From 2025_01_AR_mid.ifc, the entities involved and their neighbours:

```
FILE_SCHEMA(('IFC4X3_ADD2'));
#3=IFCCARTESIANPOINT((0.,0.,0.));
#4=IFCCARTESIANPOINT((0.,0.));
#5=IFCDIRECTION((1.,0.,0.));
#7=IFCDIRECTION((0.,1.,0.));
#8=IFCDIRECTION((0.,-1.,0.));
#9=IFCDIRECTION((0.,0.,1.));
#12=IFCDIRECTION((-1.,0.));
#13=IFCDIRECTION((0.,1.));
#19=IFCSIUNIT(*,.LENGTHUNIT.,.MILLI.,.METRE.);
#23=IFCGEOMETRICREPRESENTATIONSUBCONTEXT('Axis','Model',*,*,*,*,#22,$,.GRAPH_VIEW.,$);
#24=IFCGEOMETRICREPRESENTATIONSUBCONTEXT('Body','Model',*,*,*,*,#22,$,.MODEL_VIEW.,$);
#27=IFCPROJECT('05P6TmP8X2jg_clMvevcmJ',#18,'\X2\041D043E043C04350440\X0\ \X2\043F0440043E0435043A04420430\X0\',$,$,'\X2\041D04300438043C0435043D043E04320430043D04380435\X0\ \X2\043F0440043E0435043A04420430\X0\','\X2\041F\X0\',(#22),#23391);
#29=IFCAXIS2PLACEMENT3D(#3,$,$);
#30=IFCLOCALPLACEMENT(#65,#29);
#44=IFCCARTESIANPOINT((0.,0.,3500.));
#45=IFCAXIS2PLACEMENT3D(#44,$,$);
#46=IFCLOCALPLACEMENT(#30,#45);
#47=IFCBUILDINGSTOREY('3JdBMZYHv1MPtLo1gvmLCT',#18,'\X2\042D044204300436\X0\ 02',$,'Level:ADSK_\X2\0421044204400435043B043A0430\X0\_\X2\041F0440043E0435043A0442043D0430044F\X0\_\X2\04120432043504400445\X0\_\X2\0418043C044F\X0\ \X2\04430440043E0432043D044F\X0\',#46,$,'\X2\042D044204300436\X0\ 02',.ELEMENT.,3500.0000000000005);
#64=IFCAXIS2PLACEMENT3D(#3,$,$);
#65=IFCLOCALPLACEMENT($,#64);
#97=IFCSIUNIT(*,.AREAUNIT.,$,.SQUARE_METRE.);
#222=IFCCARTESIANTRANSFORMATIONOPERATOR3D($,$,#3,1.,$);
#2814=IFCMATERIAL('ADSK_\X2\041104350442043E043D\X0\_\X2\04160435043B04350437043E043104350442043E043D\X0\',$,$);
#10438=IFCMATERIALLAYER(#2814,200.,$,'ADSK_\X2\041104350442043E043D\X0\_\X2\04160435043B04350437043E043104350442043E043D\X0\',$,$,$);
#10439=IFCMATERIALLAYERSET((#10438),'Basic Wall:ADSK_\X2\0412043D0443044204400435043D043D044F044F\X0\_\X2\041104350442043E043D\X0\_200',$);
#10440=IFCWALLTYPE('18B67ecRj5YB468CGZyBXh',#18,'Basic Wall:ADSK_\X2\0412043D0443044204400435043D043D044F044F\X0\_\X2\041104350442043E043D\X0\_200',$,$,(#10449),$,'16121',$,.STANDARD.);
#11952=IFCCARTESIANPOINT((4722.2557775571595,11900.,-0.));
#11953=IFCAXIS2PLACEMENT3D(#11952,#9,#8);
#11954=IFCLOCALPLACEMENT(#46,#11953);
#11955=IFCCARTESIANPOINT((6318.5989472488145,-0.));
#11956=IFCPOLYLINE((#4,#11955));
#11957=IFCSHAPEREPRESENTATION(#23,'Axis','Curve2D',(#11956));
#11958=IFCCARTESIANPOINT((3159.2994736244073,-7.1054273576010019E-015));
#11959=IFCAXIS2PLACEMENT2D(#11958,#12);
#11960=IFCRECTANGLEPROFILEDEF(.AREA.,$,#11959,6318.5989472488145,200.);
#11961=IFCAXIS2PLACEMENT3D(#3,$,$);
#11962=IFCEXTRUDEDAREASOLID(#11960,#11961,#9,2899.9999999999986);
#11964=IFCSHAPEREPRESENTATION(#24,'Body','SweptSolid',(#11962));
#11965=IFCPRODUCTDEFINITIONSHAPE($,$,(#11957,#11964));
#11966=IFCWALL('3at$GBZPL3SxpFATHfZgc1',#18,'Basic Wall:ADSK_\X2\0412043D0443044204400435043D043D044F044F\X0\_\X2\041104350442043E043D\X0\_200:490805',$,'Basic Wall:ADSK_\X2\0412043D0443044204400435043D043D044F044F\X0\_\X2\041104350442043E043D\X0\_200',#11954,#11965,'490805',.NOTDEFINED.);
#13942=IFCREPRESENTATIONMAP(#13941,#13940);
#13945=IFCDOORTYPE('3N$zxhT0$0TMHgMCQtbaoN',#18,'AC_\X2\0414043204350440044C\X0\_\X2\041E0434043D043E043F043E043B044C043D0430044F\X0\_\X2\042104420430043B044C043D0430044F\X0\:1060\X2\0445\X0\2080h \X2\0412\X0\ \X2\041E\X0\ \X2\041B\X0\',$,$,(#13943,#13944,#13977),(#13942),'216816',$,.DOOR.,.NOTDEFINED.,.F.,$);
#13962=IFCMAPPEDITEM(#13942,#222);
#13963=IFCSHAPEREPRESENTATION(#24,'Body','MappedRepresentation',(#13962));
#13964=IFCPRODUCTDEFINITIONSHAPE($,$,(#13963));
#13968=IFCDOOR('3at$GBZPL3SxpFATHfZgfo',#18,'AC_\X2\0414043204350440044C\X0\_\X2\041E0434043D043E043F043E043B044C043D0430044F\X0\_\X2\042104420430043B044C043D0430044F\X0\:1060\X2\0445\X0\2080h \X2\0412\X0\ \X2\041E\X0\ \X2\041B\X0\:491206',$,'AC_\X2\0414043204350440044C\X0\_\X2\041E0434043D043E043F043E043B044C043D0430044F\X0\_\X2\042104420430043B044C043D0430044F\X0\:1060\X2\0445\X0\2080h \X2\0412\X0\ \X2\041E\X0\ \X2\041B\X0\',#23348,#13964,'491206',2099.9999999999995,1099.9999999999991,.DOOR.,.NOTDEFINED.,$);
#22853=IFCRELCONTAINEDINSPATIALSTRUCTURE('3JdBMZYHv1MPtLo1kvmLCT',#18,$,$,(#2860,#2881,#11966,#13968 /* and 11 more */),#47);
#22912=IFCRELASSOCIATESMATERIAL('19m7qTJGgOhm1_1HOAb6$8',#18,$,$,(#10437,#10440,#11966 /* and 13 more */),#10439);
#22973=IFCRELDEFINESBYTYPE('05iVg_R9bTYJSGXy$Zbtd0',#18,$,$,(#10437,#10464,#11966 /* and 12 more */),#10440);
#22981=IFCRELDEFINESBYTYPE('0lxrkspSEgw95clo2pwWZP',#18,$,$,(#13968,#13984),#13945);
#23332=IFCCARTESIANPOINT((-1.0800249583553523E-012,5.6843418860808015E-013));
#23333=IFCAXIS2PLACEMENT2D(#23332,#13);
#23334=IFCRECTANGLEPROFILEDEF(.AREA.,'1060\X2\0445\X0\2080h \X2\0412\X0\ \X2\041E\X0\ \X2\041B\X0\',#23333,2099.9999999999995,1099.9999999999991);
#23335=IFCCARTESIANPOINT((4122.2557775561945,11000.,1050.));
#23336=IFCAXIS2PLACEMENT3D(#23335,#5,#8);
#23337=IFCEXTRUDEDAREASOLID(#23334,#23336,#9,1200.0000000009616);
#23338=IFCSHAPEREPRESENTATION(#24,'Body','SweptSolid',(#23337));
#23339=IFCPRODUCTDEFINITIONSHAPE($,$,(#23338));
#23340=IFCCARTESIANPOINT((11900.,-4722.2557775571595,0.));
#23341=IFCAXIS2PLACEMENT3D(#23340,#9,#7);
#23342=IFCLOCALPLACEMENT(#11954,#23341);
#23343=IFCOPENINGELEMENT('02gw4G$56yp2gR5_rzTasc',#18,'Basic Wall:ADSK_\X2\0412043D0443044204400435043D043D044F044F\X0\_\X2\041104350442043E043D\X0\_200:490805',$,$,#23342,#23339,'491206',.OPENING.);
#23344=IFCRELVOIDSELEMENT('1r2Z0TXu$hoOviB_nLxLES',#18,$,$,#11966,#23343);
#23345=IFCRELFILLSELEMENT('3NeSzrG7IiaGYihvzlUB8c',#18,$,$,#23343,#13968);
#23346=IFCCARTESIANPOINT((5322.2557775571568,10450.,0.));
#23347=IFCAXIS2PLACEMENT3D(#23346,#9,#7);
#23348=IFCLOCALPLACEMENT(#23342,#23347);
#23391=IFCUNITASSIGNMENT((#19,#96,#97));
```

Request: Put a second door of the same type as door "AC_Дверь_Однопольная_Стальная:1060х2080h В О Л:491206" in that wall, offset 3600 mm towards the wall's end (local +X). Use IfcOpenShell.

```python
import ifcopenshell
import ifcopenshell.api.feature
import ifcopenshell.api.geometry
import ifcopenshell.api.root
import ifcopenshell.geom
import ifcopenshell.util.element
import ifcopenshell.util.placement
import ifcopenshell.util.shape
import ifcopenshell.util.unit

model = ifcopenshell.open("2025_01_AR_mid.ifc")
unit_scale = ifcopenshell.util.unit.calculate_unit_scale(model)
settings = ifcopenshell.geom.settings()


def volume(element):
    """Net volume in cubic metres, openings subtracted."""
    shape = ifcopenshell.geom.create_shape(settings, element)
    return ifcopenshell.util.shape.get_volume(shape.geometry)


def reuse_history(source, copy):
    """copy_class also copies each property set's owner history, people and application; keep the originals."""
    for rel in copy.IsDefinedBy:
        if rel.is_a("IfcRelDefinesByProperties") and (history := rel.RelatingPropertyDefinition.OwnerHistory):
            rel.RelatingPropertyDefinition.OwnerHistory = source.OwnerHistory
            ifcopenshell.util.element.remove_deep2(model, history)


door = model.by_guid("3at$GBZPL3SxpFATHfZgfo")
opening = door.FillsVoids[0].RelatingOpeningElement
wall = opening.VoidsElements[0].RelatingBuildingElement
before = volume(wall)
shift = ifcopenshell.util.placement.get_local_placement(wall.ObjectPlacement)[:3, 0] * 3.6 / unit_scale

# copy_class copies the void relationship, type, container and properties, but no geometry.
new_opening = ifcopenshell.api.root.copy_class(model, product=opening)
new_opening.Representation = ifcopenshell.util.element.copy_deep(
    model, opening.Representation, exclude=["IfcGeometricRepresentationContext", "IfcRepresentationMap"]
)
new_opening.Name = "Basic Wall:ADSK_Внутренняя_Бетон_200"
new_opening.Tag = None
new_door = ifcopenshell.api.root.copy_class(model, product=door)
new_door.Representation = ifcopenshell.util.element.copy_deep(
    model, door.Representation, exclude=["IfcGeometricRepresentationContext", "IfcRepresentationMap"]
)
new_door.Name = "AC_Дверь_Однопольная_Стальная:1060х2080h В О Л"
new_door.Tag = None
reuse_history(door, new_door)
ifcopenshell.api.feature.add_filling(model, opening=new_opening, element=new_door)

for old, new in ((opening, new_opening), (door, new_door)):
    matrix = ifcopenshell.util.placement.get_local_placement(old.ObjectPlacement)
    matrix[:3, 3] += shift
    ifcopenshell.api.geometry.edit_object_placement(model, product=new, matrix=matrix, is_si=False)

after = volume(wall)

print(f"wall volume {before:.3f} -> {after:.3f} m3")

model.write("2025_01_AR_mid_rev.ifc")
```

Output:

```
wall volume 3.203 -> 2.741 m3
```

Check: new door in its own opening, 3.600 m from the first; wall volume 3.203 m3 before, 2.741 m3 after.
